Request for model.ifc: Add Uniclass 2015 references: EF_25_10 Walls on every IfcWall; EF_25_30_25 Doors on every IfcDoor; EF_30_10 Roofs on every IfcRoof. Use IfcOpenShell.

First a look at what the model holds.

```python
import ifcopenshell

model = ifcopenshell.open("model.ifc")
print(model.schema)
print("classifications:", [c.Name for c in model.by_type("IfcClassification")])
for ifc_class in ("IfcDoor", "IfcRoof", "IfcStair", "IfcWall", "IfcWindow"):
    print(ifc_class, len(model.by_type(ifc_class)))
```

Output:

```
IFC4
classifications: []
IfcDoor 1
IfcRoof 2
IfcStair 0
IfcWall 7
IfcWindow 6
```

```python
import ifcopenshell
import ifcopenshell.api.classification

model = ifcopenshell.open("model.ifc")

system = ifcopenshell.api.classification.add_classification(model, classification="Uniclass 2015")

codes = {
    "IfcWall": ("EF_25_10", "Walls"),
    "IfcDoor": ("EF_25_30_25", "Doors"),
    "IfcRoof": ("EF_30_10", "Roofs"),
}
for ifc_class, (code, name) in codes.items():
    products = model.by_type(ifc_class)
    ifcopenshell.api.classification.add_reference(
        model, products=products, classification=system, identification=code, name=name
    )
    print(code, len(products))

model.write("model_updated.ifc")
```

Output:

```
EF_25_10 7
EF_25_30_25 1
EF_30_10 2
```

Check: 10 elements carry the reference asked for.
